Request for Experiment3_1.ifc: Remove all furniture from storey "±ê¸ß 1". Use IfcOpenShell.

First a look at what the model holds.

```python
import ifcopenshell
import ifcopenshell.util.element

model = ifcopenshell.open("Experiment3_1.ifc")
print(model.schema)
storey = next(s for s in model.by_type("IfcBuildingStorey") if s.Name == "±ê¸ß 1")
furniture = [e for e in ifcopenshell.util.element.get_decomposition(storey) if e.is_a("IfcFurnishingElement")]
seen = {}
for e in furniture:
    element_type = ifcopenshell.util.element.get_type(e)
    name = element_type.Name if element_type not in (None, e) else None
    seen[name] = seen.get(name, 0) + 1
for name, count in sorted(seen.items(), key=str):
    print(count, "x", name)
```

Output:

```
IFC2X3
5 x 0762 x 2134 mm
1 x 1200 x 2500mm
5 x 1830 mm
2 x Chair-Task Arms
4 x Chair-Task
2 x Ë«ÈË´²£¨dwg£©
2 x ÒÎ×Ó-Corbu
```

```python
import ifcopenshell
import ifcopenshell.api.root
import ifcopenshell.util.element

model = ifcopenshell.open("Experiment3_1.ifc")

storey = next(s for s in model.by_type("IfcBuildingStorey") if s.Name == "±ê¸ß 1")
furniture = [e for e in ifcopenshell.util.element.get_decomposition(storey) if e.is_a("IfcFurnishingElement")]

for e in furniture:
    ifcopenshell.api.root.remove_product(model, product=e)
print(len(furniture), "removed")

model.write("Experiment3_1_edited.ifc")
```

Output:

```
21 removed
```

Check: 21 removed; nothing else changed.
